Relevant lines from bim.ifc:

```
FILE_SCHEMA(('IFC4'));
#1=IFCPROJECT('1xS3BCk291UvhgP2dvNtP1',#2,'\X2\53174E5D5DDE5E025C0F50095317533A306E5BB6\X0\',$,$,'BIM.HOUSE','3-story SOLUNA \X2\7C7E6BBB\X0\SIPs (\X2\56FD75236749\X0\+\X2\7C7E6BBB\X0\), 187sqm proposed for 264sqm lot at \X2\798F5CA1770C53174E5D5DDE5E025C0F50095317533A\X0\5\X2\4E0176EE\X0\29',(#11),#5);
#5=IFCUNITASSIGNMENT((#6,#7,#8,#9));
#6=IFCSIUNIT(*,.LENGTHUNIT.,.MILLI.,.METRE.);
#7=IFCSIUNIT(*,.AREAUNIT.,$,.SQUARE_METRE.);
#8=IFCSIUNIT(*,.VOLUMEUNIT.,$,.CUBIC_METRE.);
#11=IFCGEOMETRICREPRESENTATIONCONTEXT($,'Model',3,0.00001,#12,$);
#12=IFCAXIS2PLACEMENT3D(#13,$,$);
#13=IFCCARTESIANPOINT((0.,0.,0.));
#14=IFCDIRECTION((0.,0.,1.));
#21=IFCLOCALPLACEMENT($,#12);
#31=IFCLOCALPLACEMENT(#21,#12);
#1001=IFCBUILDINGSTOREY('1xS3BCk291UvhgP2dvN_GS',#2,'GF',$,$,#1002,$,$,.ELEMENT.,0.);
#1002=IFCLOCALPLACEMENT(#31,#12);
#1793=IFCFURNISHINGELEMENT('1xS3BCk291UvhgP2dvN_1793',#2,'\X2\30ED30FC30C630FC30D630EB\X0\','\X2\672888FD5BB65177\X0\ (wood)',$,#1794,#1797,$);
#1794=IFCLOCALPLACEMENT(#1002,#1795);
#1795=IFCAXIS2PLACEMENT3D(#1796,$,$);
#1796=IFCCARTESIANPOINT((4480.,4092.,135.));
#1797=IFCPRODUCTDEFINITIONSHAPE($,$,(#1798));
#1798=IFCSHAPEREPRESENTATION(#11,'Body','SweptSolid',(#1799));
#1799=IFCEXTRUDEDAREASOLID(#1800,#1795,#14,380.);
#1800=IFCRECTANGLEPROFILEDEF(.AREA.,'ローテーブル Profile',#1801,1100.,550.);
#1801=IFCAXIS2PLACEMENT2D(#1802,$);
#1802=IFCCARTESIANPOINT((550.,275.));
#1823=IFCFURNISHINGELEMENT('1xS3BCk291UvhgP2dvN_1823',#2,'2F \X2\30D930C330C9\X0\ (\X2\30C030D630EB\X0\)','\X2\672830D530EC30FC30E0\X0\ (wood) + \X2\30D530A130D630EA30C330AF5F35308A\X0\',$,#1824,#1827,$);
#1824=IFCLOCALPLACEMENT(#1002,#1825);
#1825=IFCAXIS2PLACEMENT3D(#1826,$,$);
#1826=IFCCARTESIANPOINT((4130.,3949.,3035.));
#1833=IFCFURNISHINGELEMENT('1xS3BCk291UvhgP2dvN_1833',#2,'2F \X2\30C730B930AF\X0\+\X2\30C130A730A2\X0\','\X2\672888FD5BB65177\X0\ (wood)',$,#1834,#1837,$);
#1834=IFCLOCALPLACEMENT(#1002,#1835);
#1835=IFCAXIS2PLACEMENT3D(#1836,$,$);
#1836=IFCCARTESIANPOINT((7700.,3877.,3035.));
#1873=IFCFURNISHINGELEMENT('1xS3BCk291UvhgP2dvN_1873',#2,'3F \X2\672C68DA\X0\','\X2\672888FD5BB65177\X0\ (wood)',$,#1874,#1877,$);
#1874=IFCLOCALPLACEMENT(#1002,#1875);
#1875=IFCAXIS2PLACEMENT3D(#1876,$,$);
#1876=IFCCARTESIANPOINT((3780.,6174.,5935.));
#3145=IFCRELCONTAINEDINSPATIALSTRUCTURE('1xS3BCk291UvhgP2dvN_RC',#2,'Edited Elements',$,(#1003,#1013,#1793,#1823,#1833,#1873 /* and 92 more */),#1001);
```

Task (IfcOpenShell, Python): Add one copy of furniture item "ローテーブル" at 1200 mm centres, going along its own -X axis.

```python
import ifcopenshell
import ifcopenshell.api.geometry
import ifcopenshell.api.root
import ifcopenshell.util.element
import ifcopenshell.util.placement

model = ifcopenshell.open("bim.ifc")


def reuse_history(source, copy):
    """copy_class also copies each property set's owner history, people and application; keep the originals."""
    for rel in copy.IsDefinedBy:
        if rel.is_a("IfcRelDefinesByProperties") and (history := rel.RelatingPropertyDefinition.OwnerHistory):
            rel.RelatingPropertyDefinition.OwnerHistory = source.OwnerHistory
            ifcopenshell.util.element.remove_deep2(model, history)


source = model.by_id(1793)
base = ifcopenshell.util.placement.get_local_placement(source.ObjectPlacement)
step = -base[:3, 0] * 1200.0

for i in range(1, 2):
    copy = ifcopenshell.api.root.copy_class(model, product=source)
    copy.Representation = ifcopenshell.util.element.copy_deep(
        model, source.Representation, exclude=["IfcGeometricRepresentationContext", "IfcRepresentationMap"]
    )
    reuse_history(source, copy)
    matrix = base.copy()
    matrix[:3, 3] += i * step
    print("added at", matrix[:3, 3].round(3) + 0.0)
    ifcopenshell.api.geometry.edit_object_placement(model, product=copy, matrix=matrix, is_si=False)

model.write("bim_rev.ifc")
```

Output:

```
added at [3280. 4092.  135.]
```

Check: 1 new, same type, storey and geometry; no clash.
